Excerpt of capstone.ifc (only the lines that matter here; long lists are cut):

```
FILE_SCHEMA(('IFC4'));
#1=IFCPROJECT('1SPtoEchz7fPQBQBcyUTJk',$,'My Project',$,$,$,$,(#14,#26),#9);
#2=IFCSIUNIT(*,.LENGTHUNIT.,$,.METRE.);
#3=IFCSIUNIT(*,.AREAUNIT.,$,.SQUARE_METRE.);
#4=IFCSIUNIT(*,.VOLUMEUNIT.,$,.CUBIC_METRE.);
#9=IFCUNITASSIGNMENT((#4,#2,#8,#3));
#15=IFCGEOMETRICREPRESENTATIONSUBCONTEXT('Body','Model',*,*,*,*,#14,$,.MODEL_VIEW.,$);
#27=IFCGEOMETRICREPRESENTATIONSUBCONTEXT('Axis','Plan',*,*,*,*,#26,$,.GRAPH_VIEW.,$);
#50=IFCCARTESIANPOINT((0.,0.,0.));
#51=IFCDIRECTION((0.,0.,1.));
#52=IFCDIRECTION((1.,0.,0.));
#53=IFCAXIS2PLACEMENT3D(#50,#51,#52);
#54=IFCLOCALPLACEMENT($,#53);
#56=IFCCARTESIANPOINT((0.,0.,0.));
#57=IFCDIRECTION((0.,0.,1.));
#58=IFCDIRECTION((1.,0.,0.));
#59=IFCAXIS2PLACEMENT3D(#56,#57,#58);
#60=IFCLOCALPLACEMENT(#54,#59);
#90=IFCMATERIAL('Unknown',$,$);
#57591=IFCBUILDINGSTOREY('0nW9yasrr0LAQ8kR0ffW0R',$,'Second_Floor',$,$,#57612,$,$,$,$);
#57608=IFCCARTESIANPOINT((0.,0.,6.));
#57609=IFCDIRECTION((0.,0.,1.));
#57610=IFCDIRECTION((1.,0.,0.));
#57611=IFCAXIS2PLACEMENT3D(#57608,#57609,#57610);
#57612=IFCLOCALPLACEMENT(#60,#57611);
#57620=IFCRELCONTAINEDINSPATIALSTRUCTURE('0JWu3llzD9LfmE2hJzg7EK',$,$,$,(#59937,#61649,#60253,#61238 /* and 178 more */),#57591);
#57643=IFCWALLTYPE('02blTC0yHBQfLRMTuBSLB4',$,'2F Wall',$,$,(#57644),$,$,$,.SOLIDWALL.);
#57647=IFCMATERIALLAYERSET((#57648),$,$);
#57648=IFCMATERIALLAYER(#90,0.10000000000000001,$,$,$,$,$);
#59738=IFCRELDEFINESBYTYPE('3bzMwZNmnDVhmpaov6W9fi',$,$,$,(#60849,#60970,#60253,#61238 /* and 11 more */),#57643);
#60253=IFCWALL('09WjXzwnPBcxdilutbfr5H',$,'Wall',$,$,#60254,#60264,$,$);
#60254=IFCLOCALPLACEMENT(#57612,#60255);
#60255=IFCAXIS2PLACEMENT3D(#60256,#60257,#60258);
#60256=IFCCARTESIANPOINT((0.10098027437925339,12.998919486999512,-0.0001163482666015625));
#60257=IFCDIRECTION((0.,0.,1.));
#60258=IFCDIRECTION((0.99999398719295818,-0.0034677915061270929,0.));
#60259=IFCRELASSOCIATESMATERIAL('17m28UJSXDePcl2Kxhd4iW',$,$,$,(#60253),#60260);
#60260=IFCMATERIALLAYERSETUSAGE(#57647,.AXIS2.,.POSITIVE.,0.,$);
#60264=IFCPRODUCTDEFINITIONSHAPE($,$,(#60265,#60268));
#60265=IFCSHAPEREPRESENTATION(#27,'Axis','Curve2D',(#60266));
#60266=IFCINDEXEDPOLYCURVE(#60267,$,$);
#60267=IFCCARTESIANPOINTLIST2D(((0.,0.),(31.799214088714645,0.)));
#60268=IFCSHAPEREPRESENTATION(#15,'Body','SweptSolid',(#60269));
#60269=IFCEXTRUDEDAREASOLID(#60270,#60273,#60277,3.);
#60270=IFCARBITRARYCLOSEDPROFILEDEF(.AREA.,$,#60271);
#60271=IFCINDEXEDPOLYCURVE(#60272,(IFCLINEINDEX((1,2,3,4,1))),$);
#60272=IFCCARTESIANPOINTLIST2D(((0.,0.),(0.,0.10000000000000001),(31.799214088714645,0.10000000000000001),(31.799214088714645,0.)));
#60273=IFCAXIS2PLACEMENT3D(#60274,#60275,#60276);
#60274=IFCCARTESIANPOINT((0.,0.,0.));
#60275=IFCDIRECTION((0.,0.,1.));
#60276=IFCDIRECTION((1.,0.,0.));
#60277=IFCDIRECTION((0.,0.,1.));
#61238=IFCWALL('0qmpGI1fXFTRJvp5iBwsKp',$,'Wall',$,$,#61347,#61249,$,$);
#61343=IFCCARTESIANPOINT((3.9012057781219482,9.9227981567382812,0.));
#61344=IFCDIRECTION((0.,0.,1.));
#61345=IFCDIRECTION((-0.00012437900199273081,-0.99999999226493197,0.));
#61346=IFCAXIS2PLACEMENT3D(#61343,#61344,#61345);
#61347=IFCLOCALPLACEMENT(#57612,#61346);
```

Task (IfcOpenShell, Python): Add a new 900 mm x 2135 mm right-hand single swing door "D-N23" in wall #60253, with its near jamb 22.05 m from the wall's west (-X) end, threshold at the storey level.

```python
import numpy as np
import ifcopenshell
import ifcopenshell.api.feature
import ifcopenshell.api.geometry
import ifcopenshell.api.root
import ifcopenshell.api.spatial
import ifcopenshell.geom
import ifcopenshell.util.element
import ifcopenshell.util.placement
import ifcopenshell.util.representation
import ifcopenshell.util.shape
import ifcopenshell.util.unit

model = ifcopenshell.open("capstone.ifc")
unit_scale = ifcopenshell.util.unit.calculate_unit_scale(model)
settings = ifcopenshell.geom.settings()


def volume(element):
    """Net volume in cubic metres, openings subtracted."""
    shape = ifcopenshell.geom.create_shape(settings, element)
    return ifcopenshell.util.shape.get_volume(shape.geometry)


wall = model.by_guid("09WjXzwnPBcxdilutbfr5H")
storey = ifcopenshell.util.element.get_container(wall, ifc_class="IfcBuildingStorey")
context = ifcopenshell.util.representation.get_context(model, "Model", "Body", "MODEL_VIEW")
before = volume(wall)

width, height, from_end, sill = 0.9, 2.135, 22.05, 0.0  # metres

# The wall runs along its own X axis, and the end named is its -X end.
wall_shape = ifcopenshell.geom.create_shape(settings, wall)
x, y, z = ifcopenshell.util.shape.get_vertices(wall_shape.geometry).T
start = x.min() + from_end
face, thickness = float(y.min()), float(y.max() - y.min())
wall_matrix = ifcopenshell.util.placement.get_local_placement(wall.ObjectPlacement)
level = ifcopenshell.util.placement.get_local_placement(storey.ObjectPlacement)[2, 3]


def in_wall(x, y):
    """Placement at x, y metres in the wall's axes, at sill height."""
    matrix = wall_matrix.copy()
    matrix[:, 3] = wall_matrix @ np.array([x / unit_scale, y / unit_scale, 0.0, 1.0])
    matrix[2, 3] = level + sill / unit_scale
    return matrix


# Opening: a box that overshoots both wall faces by 50 mm.
opening = ifcopenshell.api.root.create_entity(model, ifc_class="IfcOpeningElement", predefined_type="OPENING")
box = ifcopenshell.api.geometry.add_wall_representation(
    model, context=context, length=width, height=height, thickness=thickness + 0.1
)
ifcopenshell.api.geometry.assign_representation(model, product=opening, representation=box)
ifcopenshell.api.geometry.edit_object_placement(model, product=opening, matrix=in_wall(start, face - 0.05), is_si=False)
ifcopenshell.api.feature.add_feature(model, feature=opening, element=wall)

door = ifcopenshell.api.root.create_entity(model, ifc_class="IfcDoor", name="D-N23", predefined_type="DOOR")
door.OverallWidth, door.OverallHeight = width / unit_scale, height / unit_scale
door.OperationType = "SINGLE_SWING_RIGHT"
body = ifcopenshell.api.geometry.add_door_representation(
    model,
    context=context,
    overall_width=door.OverallWidth,
    overall_height=door.OverallHeight,
    operation_type="SINGLE_SWING_RIGHT",
    lining_properties={"LiningDepth": thickness / unit_scale, "ThresholdDepth": thickness / unit_scale},
)
ifcopenshell.api.geometry.assign_representation(model, product=door, representation=body)
ifcopenshell.api.spatial.assign_container(model, products=[door], relating_structure=storey)
ifcopenshell.api.feature.add_filling(model, opening=opening, element=door)

# The lining spans the wall, so the door starts at the wall face.
ifcopenshell.api.geometry.edit_object_placement(model, product=door, matrix=in_wall(start, face), is_si=False)

after = volume(wall)

print(f"wall volume {before:.3f} -> {after:.3f} m3")

model.write("capstone-out.ifc")
```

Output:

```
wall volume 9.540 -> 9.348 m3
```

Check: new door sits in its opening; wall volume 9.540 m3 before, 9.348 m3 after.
